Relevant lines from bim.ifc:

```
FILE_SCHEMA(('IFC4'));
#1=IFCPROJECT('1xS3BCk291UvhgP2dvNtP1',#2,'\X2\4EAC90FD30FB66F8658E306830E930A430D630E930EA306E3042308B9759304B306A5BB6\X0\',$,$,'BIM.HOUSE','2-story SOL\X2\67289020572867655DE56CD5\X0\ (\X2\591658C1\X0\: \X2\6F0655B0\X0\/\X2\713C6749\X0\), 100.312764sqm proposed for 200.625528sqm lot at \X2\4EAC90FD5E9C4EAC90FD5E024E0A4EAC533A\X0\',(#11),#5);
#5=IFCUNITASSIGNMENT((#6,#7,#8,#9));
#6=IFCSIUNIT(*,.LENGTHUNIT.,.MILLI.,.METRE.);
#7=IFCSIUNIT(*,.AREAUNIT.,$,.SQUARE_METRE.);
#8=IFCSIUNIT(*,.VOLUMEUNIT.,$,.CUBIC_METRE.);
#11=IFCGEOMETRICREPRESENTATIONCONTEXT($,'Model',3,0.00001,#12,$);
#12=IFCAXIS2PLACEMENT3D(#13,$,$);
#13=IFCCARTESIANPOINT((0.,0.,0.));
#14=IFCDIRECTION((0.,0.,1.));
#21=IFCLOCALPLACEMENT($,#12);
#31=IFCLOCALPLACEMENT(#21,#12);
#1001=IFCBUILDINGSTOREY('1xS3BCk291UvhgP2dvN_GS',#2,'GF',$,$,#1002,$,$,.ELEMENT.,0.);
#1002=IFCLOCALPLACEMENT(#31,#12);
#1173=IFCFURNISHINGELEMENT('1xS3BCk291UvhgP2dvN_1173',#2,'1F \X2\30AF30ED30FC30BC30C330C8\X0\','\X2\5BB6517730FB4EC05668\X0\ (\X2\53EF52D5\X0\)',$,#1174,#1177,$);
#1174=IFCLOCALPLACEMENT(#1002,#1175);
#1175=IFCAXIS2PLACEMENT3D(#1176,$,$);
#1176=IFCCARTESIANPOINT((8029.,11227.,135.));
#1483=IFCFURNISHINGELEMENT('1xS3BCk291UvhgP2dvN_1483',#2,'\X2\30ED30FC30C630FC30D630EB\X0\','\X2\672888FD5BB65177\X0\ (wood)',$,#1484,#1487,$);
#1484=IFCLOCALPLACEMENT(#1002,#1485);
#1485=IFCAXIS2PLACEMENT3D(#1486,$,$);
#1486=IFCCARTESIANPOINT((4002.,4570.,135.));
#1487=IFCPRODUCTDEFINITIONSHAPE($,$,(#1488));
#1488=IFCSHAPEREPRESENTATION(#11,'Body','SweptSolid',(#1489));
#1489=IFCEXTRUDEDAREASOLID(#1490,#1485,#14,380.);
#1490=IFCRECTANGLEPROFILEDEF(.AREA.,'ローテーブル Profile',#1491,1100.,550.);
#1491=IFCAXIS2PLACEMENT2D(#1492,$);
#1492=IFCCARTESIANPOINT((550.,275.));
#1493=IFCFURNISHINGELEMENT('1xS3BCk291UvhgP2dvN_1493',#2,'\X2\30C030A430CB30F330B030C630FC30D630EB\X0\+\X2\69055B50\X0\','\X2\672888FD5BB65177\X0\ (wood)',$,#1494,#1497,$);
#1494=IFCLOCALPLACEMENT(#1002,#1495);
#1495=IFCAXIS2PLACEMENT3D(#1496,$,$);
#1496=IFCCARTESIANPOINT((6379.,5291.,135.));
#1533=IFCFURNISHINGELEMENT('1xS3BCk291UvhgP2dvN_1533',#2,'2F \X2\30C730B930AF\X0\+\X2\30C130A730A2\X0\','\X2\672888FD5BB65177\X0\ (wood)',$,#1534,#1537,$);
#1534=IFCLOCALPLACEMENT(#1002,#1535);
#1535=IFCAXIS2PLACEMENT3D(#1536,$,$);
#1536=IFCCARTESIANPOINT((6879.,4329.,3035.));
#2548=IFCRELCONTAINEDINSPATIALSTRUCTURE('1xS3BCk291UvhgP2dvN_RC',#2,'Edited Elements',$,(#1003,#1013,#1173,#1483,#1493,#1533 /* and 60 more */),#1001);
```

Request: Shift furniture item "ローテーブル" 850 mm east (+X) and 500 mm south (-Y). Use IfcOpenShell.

```python
import ifcopenshell
import ifcopenshell.api.geometry
import ifcopenshell.util.placement

model = ifcopenshell.open("bim.ifc")

item = model.by_id(1483)
matrix = ifcopenshell.util.placement.get_local_placement(item.ObjectPlacement)
matrix[0, 3] += 850.0
matrix[1, 3] -= 500.0
ifcopenshell.api.geometry.edit_object_placement(model, product=item, matrix=matrix, is_si=False)

print(ifcopenshell.util.placement.get_local_placement(item.ObjectPlacement).round(3) + 0.0)

model.write("bim-out.ifc")
```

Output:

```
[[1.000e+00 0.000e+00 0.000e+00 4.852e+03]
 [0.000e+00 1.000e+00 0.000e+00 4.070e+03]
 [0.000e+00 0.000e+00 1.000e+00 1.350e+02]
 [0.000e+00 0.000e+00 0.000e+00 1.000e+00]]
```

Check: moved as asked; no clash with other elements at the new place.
